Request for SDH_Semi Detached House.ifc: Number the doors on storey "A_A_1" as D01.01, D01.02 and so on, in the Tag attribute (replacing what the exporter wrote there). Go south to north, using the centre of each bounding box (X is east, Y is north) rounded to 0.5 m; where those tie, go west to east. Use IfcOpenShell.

First a look at what the model holds.

```python
import ifcopenshell
import ifcopenshell.util.element
import ifcopenshell.util.placement

model = ifcopenshell.open("SDH_Semi Detached House.ifc")
print(model.schema)
storey = next(s for s in model.by_type("IfcBuildingStorey") if s.Name == "A_A_1")
doors = [e for e in ifcopenshell.util.element.get_decomposition(storey) if e.is_a("IfcDoor")]
for e in sorted(doors, key=lambda e: e.id()):
    origin = ifcopenshell.util.placement.get_local_placement(e.ObjectPlacement)[:3, 3]
    print(e.id(), e.Tag, e.Name, origin.round(2) + 0.0, sep=" | ")
```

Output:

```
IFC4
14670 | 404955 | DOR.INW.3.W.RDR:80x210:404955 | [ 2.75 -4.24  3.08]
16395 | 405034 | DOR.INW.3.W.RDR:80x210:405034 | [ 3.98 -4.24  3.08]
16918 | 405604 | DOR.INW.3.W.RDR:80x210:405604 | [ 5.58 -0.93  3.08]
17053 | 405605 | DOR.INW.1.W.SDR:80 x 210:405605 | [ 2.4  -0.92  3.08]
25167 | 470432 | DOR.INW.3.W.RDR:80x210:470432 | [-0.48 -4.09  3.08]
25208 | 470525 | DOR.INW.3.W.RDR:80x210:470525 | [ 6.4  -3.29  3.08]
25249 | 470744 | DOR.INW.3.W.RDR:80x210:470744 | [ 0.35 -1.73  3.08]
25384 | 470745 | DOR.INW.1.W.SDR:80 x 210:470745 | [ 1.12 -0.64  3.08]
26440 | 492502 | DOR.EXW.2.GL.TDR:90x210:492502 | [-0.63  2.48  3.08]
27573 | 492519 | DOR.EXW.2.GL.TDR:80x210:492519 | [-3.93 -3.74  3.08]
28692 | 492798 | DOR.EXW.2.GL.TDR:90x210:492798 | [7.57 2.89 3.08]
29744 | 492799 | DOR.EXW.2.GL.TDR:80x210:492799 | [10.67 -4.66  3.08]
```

```python
import ifcopenshell
import ifcopenshell.geom
import ifcopenshell.util.element
import ifcopenshell.util.shape

model = ifcopenshell.open("SDH_Semi Detached House.ifc")
settings = ifcopenshell.geom.settings()
settings.set("use-world-coords", True)


def centre(element):
    shape = ifcopenshell.geom.create_shape(settings, element)
    return ifcopenshell.util.shape.get_bbox_centroid(shape.geometry)


storey = next(s for s in model.by_type("IfcBuildingStorey") if s.Name == "A_A_1")
doors = [e for e in ifcopenshell.util.element.get_decomposition(storey) if e.is_a("IfcDoor")]

# Insertion points can sit at a corner or the storey origin, so sort by the geometry (in metres).
centres = {e: centre(e) for e in doors}
doors.sort(key=lambda e: (round(centres[e][1] / 0.5), centres[e][0]))

for i, e in enumerate(doors, start=1):
    number = f"D01.{i:02d}"
    e.Tag = number
    print(e.id(), number)

model.write("SDH_Semi Detached House_v2.ifc")
```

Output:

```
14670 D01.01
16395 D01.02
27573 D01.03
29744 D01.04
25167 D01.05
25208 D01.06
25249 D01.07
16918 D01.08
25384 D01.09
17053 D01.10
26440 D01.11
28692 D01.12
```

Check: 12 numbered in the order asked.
